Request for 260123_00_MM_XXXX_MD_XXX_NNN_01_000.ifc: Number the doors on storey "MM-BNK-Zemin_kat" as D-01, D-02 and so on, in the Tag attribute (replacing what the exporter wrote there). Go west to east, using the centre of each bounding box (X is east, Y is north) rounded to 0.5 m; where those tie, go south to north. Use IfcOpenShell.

First a look at what the model holds.

```python
import ifcopenshell
import ifcopenshell.util.element
import ifcopenshell.util.placement

model = ifcopenshell.open("260123_00_MM_XXXX_MD_XXX_NNN_01_000.ifc")
print(model.schema)
storey = next(s for s in model.by_type("IfcBuildingStorey") if s.Name == "MM-BNK-Zemin_kat")
doors = [e for e in ifcopenshell.util.element.get_decomposition(storey) if e.is_a("IfcDoor")]
for e in sorted(doors, key=lambda e: e.id()):
    origin = ifcopenshell.util.placement.get_local_placement(e.ObjectPlacement)[:3, 3]
    print(e.id(), e.Tag, e.Name, origin.round(2) + 0.0, sep=" | ")
```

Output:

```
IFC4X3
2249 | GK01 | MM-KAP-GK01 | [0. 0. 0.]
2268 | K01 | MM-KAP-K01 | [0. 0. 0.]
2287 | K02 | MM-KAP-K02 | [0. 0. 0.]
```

```python
import ifcopenshell
import ifcopenshell.geom
import ifcopenshell.util.element
import ifcopenshell.util.shape

model = ifcopenshell.open("260123_00_MM_XXXX_MD_XXX_NNN_01_000.ifc")
settings = ifcopenshell.geom.settings()
settings.set("use-world-coords", True)


def centre(element):
    shape = ifcopenshell.geom.create_shape(settings, element)
    return ifcopenshell.util.shape.get_bbox_centroid(shape.geometry)


storey = next(s for s in model.by_type("IfcBuildingStorey") if s.Name == "MM-BNK-Zemin_kat")
doors = [e for e in ifcopenshell.util.element.get_decomposition(storey) if e.is_a("IfcDoor")]

# Insertion points can sit at a corner or the storey origin, so sort by the geometry (in metres).
centres = {e: centre(e) for e in doors}
doors.sort(key=lambda e: (round(centres[e][0] / 0.5), centres[e][1]))

for i, e in enumerate(doors, start=1):
    number = f"D-{i:02d}"
    e.Tag = number
    print(e.id(), number)

model.write("260123_00_MM_XXXX_MD_XXX_NNN_01_000-out.ifc")
```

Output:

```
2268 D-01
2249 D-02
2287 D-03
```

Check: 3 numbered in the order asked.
